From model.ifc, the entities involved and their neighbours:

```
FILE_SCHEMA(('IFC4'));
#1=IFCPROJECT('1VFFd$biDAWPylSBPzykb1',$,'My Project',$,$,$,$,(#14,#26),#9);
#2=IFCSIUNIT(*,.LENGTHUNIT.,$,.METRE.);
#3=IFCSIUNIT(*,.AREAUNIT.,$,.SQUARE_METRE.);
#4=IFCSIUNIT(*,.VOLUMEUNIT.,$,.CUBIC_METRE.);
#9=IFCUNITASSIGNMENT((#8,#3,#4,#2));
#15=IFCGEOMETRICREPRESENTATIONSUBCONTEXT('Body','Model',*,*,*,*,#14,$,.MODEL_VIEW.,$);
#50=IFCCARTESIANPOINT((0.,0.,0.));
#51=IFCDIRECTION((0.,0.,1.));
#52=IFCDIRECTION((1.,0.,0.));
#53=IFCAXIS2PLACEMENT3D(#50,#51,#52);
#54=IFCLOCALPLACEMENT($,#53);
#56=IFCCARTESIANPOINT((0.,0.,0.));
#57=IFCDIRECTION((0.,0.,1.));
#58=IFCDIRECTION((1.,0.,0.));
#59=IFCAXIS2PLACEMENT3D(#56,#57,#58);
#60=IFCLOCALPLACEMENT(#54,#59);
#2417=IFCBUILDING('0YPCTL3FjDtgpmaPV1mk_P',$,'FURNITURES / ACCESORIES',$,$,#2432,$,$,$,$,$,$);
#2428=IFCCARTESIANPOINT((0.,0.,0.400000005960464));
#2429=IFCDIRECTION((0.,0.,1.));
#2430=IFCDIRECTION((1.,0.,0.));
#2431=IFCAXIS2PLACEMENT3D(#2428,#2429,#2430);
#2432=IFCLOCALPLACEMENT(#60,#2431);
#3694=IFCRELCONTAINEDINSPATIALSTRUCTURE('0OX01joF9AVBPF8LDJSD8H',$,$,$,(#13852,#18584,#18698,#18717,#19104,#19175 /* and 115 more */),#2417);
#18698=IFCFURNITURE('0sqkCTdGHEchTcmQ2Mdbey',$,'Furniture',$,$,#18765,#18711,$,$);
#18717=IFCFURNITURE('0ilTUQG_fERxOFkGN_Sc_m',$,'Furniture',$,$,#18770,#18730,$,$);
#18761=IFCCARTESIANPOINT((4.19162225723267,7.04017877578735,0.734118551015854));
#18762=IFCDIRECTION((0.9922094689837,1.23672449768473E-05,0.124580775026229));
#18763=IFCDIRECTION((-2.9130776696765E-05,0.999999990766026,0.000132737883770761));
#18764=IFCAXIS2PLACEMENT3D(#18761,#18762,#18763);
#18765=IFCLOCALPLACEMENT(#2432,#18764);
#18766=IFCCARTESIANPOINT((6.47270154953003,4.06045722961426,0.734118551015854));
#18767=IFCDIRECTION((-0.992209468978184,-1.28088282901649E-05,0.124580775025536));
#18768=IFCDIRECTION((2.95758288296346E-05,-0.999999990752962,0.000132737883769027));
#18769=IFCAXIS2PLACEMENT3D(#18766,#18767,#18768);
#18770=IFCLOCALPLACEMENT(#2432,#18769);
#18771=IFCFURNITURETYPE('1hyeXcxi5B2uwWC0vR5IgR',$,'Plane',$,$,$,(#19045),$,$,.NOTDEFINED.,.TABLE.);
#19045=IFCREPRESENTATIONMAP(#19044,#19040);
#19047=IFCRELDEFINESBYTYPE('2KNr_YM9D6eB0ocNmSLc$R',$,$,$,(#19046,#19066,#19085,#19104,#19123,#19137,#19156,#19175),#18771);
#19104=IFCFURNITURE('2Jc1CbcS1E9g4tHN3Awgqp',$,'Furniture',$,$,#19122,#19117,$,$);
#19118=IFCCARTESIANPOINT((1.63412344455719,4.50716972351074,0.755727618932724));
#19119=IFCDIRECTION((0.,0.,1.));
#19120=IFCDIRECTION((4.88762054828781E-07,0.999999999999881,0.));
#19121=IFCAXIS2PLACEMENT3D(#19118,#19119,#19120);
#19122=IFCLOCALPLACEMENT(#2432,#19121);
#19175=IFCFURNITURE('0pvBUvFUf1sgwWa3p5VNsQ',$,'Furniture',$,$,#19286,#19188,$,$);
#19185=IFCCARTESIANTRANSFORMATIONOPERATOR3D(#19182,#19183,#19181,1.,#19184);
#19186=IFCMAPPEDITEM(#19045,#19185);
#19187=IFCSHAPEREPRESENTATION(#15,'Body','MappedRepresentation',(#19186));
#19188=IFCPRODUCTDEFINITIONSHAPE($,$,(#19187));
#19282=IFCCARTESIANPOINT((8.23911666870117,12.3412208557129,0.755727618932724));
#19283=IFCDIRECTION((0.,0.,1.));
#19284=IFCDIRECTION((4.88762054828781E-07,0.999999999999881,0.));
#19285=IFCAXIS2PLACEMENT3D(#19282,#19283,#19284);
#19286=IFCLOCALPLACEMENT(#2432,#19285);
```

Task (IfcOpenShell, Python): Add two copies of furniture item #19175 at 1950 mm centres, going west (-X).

```python
import numpy as np
import ifcopenshell
import ifcopenshell.api.geometry
import ifcopenshell.api.root
import ifcopenshell.util.element
import ifcopenshell.util.placement
import ifcopenshell.util.unit

model = ifcopenshell.open("model.ifc")
unit_scale = ifcopenshell.util.unit.calculate_unit_scale(model)

source = model.by_guid("0pvBUvFUf1sgwWa3p5VNsQ")
base = ifcopenshell.util.placement.get_local_placement(source.ObjectPlacement)
step = np.array([-1.0, 0.0, 0.0]) * 1.95 / unit_scale

for i in range(1, 3):
    copy = ifcopenshell.api.root.copy_class(model, product=source)
    copy.Representation = ifcopenshell.util.element.copy_deep(
        model, source.Representation, exclude=["IfcGeometricRepresentationContext", "IfcRepresentationMap"]
    )
    matrix = base.copy()
    matrix[:3, 3] += i * step
    print("added at", matrix[:3, 3].round(3) + 0.0)
    ifcopenshell.api.geometry.edit_object_placement(model, product=copy, matrix=matrix, is_si=False)

model.write("model_v2.ifc")
```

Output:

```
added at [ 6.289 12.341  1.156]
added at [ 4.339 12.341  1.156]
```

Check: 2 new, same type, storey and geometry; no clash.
